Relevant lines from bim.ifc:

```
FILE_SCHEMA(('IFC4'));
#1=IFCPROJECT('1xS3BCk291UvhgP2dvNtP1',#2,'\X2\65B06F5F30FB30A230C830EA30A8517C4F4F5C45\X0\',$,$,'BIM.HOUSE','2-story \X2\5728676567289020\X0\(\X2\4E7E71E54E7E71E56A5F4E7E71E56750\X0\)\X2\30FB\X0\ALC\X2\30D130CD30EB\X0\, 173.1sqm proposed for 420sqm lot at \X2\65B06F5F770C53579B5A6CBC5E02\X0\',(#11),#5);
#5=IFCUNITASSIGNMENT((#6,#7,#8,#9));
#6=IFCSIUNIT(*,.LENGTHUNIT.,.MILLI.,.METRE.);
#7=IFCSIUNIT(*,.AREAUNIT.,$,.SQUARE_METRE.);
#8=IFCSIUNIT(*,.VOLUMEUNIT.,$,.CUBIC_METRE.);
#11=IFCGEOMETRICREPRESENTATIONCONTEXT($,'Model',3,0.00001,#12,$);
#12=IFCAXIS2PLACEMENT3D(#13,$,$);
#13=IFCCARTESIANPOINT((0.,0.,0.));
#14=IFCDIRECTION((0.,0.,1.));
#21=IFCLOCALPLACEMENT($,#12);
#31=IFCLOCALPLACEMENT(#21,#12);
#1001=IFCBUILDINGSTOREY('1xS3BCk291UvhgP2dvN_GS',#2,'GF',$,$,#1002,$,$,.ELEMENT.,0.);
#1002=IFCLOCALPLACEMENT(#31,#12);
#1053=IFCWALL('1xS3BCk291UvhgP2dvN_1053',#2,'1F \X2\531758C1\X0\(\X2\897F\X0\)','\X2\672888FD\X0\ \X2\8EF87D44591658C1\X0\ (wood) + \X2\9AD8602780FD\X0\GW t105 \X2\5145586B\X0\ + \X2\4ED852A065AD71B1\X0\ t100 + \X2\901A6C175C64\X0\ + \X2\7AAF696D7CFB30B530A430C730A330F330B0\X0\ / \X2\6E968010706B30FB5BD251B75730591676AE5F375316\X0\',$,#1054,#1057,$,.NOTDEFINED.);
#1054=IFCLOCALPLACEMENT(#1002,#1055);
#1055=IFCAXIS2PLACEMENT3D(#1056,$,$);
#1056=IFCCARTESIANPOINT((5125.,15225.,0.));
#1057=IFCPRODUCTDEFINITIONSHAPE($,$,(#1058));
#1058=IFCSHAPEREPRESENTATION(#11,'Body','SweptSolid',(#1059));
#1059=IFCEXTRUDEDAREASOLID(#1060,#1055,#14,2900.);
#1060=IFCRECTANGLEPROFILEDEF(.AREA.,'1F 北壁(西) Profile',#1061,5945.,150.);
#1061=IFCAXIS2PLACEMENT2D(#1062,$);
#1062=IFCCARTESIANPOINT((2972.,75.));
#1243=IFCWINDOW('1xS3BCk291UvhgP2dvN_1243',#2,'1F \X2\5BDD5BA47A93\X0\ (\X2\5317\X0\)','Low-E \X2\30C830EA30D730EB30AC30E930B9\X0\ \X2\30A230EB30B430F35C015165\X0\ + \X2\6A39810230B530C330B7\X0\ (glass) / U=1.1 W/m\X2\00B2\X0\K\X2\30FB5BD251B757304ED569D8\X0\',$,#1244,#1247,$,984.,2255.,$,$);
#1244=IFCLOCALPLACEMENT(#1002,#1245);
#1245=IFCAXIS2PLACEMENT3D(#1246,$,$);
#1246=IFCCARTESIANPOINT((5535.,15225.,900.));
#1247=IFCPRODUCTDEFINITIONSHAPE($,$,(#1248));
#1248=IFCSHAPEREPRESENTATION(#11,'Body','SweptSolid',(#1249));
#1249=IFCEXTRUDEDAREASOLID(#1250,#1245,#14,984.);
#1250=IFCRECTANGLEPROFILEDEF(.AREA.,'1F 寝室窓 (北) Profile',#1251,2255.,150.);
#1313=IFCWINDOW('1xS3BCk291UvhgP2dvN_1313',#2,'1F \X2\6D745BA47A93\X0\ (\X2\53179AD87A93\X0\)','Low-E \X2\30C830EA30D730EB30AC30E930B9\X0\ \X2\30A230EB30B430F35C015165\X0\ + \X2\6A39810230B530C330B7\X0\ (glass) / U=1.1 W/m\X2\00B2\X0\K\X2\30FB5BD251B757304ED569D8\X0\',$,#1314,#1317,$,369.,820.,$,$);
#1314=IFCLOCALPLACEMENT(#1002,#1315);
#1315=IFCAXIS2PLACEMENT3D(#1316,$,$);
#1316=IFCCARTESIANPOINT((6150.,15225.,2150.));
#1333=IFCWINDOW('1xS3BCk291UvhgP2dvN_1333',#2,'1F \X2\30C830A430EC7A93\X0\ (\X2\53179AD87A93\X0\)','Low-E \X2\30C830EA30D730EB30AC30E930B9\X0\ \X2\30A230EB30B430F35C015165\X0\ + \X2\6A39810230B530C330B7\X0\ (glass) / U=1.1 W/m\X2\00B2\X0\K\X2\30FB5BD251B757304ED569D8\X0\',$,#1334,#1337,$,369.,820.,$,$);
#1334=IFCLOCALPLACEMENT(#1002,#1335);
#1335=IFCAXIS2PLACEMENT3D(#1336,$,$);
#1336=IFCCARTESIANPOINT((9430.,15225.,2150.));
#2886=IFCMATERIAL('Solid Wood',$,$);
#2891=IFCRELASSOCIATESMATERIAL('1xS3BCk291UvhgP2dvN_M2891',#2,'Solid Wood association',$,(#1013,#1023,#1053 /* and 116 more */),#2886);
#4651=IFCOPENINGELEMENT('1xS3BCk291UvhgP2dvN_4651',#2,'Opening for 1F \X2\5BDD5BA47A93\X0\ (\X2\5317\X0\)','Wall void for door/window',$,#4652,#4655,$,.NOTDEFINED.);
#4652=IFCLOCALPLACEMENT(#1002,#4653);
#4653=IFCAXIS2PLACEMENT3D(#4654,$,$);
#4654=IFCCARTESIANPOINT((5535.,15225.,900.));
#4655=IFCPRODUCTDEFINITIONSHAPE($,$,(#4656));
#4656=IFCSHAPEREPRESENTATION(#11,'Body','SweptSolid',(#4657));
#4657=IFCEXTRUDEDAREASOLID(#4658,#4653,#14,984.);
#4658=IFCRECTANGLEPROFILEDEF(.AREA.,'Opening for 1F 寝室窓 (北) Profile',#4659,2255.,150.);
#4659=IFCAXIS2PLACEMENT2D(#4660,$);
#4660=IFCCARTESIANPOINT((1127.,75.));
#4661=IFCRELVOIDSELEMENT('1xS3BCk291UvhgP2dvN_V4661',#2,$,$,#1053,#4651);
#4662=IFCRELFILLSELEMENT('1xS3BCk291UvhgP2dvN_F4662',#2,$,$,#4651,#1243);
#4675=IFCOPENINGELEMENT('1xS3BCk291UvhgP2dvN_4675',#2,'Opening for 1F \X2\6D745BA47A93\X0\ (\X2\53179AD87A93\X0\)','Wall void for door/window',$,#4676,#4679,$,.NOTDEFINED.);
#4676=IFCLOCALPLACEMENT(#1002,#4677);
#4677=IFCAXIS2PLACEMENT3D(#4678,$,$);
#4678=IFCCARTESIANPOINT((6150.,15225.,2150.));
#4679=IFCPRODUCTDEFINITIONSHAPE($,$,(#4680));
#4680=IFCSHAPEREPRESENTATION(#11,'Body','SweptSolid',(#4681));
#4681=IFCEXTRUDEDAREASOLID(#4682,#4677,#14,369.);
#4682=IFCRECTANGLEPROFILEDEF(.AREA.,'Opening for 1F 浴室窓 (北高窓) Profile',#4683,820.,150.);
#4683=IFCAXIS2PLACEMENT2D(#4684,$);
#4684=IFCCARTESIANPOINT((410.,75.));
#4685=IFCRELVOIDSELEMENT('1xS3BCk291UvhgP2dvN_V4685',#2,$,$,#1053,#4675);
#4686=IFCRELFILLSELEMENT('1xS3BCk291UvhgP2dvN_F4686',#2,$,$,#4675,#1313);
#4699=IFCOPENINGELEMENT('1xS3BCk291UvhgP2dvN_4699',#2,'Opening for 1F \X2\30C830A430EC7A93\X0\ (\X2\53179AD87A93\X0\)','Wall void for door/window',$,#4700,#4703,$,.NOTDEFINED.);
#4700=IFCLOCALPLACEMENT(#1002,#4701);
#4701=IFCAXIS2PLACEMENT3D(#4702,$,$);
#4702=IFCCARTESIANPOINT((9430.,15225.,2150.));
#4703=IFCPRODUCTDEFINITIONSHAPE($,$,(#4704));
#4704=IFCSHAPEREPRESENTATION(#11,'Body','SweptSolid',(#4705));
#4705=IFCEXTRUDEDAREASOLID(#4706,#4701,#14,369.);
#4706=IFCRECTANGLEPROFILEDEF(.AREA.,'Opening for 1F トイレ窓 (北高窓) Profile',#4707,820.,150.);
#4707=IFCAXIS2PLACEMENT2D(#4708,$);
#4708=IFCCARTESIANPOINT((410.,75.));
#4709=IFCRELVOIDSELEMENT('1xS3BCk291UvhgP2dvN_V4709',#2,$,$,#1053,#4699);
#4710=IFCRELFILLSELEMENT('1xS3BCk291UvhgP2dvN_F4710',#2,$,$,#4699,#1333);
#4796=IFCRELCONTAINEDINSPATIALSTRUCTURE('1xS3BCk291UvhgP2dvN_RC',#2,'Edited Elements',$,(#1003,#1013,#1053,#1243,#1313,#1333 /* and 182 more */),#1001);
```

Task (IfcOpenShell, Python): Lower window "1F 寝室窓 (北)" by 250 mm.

```python
import numpy as np
import ifcopenshell
import ifcopenshell.api.geometry
import ifcopenshell.util.placement
import ifcopenshell.util.unit

model = ifcopenshell.open("bim.ifc")
unit_scale = ifcopenshell.util.unit.calculate_unit_scale(model)

window = model.by_guid("1xS3BCk291UvhgP2dvN_1243")
opening = window.FillsVoids[0].RelatingOpeningElement
dz = -0.25 / unit_scale

shift = np.array([0.0, 0.0, dz])
# The window is not placed relative to its opening, so move both.
for product in (opening, window):
    matrix = ifcopenshell.util.placement.get_local_placement(product.ObjectPlacement)
    matrix[:3, 3] += shift
    ifcopenshell.api.geometry.edit_object_placement(model, product=product, matrix=matrix, is_si=False)

print(f"moved by {dz * unit_scale:+.3f} m")

model.write("bim_edited.ifc")
```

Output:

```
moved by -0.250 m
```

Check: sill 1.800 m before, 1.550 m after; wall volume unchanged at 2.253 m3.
